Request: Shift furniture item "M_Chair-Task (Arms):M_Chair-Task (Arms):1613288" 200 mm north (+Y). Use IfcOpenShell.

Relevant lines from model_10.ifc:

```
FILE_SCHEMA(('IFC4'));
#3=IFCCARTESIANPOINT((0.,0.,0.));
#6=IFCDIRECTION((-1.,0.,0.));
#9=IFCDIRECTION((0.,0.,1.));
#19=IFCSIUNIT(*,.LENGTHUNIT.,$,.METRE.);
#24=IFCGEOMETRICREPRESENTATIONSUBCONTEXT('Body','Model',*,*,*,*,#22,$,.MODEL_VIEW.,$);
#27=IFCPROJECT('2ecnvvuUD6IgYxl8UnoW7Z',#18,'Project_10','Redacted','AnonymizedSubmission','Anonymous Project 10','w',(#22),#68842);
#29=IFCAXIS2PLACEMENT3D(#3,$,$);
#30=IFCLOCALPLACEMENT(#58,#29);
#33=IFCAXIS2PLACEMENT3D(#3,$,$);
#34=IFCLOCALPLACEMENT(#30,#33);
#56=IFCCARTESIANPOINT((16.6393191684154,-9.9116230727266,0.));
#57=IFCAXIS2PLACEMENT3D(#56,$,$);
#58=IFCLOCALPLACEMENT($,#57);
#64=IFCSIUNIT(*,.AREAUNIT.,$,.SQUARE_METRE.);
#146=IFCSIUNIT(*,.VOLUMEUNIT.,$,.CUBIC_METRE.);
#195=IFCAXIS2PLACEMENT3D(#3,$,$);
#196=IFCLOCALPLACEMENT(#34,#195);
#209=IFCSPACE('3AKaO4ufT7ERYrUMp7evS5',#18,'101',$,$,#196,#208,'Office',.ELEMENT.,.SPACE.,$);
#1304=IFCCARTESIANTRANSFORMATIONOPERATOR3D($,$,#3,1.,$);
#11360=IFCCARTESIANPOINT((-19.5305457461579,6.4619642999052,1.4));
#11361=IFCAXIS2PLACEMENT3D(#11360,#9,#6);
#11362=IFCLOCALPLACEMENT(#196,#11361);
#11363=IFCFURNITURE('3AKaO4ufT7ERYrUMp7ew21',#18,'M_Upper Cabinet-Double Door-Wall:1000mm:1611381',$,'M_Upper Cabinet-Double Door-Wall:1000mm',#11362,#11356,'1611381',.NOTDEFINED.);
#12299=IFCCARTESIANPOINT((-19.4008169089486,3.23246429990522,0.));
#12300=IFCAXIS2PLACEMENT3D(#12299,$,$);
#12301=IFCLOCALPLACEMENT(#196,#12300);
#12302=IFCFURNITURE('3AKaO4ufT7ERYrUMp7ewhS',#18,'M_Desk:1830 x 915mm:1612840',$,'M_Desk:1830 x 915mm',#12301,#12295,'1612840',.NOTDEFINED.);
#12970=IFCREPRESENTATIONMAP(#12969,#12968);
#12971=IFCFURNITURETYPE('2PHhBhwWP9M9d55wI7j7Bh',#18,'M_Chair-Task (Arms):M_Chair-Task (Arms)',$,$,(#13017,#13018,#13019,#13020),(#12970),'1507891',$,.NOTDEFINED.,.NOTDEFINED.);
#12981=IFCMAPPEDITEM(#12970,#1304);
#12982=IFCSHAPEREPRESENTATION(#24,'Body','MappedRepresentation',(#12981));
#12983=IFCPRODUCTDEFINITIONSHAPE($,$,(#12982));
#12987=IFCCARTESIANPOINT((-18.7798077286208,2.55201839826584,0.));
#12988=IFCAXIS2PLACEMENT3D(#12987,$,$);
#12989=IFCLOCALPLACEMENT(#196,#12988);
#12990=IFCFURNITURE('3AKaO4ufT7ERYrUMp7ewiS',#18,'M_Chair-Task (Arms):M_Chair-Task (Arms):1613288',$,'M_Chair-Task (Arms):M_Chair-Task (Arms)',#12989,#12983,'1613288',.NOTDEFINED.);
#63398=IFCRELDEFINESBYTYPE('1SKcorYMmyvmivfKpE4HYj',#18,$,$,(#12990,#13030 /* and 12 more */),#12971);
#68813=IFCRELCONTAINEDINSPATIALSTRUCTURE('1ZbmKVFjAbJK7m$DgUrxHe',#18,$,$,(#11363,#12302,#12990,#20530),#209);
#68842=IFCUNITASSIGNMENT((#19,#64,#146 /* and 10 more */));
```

```python
import ifcopenshell
import ifcopenshell.api.geometry
import ifcopenshell.util.placement
import ifcopenshell.util.unit

model = ifcopenshell.open("model_10.ifc")
unit_scale = ifcopenshell.util.unit.calculate_unit_scale(model)

item = model.by_guid("3AKaO4ufT7ERYrUMp7ewiS")
matrix = ifcopenshell.util.placement.get_local_placement(item.ObjectPlacement)
matrix[1, 3] += 0.2 / unit_scale
ifcopenshell.api.geometry.edit_object_placement(model, product=item, matrix=matrix, is_si=False)

print(ifcopenshell.util.placement.get_local_placement(item.ObjectPlacement).round(3) + 0.0)

model.write("model_10_edited.ifc")
```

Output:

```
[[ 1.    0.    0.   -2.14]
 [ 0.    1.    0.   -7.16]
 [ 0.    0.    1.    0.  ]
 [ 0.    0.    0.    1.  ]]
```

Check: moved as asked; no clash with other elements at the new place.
